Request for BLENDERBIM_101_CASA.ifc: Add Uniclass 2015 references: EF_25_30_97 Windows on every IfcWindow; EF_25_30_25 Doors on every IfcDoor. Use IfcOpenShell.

First a look at what the model holds.

```python
import ifcopenshell

model = ifcopenshell.open("BLENDERBIM_101_CASA.ifc")
print(model.schema)
print("classifications:", [c.Name for c in model.by_type("IfcClassification")])
for ifc_class in ("IfcDoor", "IfcRoof", "IfcStair", "IfcWall", "IfcWindow"):
    print(ifc_class, len(model.by_type(ifc_class)))
```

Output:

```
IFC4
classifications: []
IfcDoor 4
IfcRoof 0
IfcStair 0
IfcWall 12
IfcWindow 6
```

```python
import ifcopenshell
import ifcopenshell.api.classification

model = ifcopenshell.open("BLENDERBIM_101_CASA.ifc")

system = ifcopenshell.api.classification.add_classification(model, classification="Uniclass 2015")

codes = {
    "IfcWindow": ("EF_25_30_97", "Windows"),
    "IfcDoor": ("EF_25_30_25", "Doors"),
}
for ifc_class, (code, name) in codes.items():
    products = model.by_type(ifc_class)
    ifcopenshell.api.classification.add_reference(
        model, products=products, classification=system, identification=code, name=name
    )
    print(code, len(products))

model.write("BLENDERBIM_101_CASA_updated.ifc")
```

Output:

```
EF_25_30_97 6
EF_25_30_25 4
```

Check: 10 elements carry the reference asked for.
